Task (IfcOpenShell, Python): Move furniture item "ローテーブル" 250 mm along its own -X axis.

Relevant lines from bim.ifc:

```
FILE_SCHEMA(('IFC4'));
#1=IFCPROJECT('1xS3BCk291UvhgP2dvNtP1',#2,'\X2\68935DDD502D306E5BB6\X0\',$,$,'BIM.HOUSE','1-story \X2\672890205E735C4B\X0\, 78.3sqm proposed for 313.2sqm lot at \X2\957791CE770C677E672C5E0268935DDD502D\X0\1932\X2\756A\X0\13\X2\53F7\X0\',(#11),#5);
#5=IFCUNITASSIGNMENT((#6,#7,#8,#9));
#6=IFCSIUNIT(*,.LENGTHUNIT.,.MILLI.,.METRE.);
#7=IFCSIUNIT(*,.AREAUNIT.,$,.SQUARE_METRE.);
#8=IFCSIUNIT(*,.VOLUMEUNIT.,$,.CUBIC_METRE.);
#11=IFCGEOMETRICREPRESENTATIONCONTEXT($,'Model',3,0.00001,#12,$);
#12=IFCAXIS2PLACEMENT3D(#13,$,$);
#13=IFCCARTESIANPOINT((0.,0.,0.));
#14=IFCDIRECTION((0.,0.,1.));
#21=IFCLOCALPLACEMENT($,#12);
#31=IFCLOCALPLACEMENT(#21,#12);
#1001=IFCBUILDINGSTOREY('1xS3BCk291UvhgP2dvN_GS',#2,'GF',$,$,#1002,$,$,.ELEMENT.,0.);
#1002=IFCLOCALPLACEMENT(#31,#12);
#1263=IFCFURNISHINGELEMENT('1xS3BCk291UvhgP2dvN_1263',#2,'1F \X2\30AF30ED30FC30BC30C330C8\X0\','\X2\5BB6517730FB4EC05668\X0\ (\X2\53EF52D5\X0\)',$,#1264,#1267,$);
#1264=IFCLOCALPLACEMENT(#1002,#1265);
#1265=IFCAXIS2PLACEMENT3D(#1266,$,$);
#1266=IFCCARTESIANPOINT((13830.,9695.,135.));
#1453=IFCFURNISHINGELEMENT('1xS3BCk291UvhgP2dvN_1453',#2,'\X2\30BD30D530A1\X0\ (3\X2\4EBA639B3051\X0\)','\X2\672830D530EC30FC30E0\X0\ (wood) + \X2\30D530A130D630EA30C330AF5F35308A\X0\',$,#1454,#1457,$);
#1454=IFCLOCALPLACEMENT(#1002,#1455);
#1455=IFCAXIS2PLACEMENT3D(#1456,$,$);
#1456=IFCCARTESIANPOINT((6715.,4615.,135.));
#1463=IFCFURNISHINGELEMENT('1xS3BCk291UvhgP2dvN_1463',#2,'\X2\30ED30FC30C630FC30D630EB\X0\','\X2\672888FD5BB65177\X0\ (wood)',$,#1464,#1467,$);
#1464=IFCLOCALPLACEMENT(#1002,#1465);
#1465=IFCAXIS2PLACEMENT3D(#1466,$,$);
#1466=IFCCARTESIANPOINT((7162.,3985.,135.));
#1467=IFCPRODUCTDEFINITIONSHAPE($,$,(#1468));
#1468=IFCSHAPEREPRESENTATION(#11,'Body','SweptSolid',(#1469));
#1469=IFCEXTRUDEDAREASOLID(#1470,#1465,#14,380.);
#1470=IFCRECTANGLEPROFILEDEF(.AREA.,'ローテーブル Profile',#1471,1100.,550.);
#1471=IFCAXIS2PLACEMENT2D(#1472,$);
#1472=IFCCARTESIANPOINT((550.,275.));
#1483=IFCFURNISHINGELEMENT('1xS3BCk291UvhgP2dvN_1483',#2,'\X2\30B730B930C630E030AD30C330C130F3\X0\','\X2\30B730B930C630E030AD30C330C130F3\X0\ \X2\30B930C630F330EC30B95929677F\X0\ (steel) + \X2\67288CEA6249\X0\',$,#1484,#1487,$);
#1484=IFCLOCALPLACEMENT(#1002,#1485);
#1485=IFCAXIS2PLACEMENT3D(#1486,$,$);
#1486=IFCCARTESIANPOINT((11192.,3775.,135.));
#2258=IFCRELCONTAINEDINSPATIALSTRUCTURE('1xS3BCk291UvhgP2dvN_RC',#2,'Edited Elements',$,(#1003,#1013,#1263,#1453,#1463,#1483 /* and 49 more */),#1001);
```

```python
import ifcopenshell
import ifcopenshell.api.geometry
import ifcopenshell.util.placement

model = ifcopenshell.open("bim.ifc")

item = model.by_guid("1xS3BCk291UvhgP2dvN_1463")
matrix = ifcopenshell.util.placement.get_local_placement(item.ObjectPlacement)
matrix[:3, 3] -= matrix[:3, 0] * 250.0
ifcopenshell.api.geometry.edit_object_placement(model, product=item, matrix=matrix, is_si=False)

print(ifcopenshell.util.placement.get_local_placement(item.ObjectPlacement).round(3) + 0.0)

model.write("bim_v2.ifc")
```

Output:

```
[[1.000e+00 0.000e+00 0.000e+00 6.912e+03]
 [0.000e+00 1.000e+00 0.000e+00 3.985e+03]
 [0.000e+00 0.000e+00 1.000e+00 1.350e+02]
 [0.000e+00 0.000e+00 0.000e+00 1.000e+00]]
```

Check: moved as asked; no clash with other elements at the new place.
